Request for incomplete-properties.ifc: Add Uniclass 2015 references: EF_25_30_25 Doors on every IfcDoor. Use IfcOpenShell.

First a look at what the model holds.

```python
import ifcopenshell

model = ifcopenshell.open("incomplete-properties.ifc")
print(model.schema)
print("classifications:", [c.Name for c in model.by_type("IfcClassification")])
for ifc_class in ("IfcDoor", "IfcRoof", "IfcStair", "IfcWall", "IfcWindow"):
    print(ifc_class, len(model.by_type(ifc_class)))
```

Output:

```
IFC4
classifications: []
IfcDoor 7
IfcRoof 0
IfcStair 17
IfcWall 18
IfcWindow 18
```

```python
import ifcopenshell
import ifcopenshell.api.classification

model = ifcopenshell.open("incomplete-properties.ifc")

system = ifcopenshell.api.classification.add_classification(model, classification="Uniclass 2015")

codes = {
    "IfcDoor": ("EF_25_30_25", "Doors"),
}
for ifc_class, (code, name) in codes.items():
    products = model.by_type(ifc_class)
    ifcopenshell.api.classification.add_reference(
        model, products=products, classification=system, identification=code, name=name
    )
    print(code, len(products))

model.write("incomplete-properties_rev.ifc")
```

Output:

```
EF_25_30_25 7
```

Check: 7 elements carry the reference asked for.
